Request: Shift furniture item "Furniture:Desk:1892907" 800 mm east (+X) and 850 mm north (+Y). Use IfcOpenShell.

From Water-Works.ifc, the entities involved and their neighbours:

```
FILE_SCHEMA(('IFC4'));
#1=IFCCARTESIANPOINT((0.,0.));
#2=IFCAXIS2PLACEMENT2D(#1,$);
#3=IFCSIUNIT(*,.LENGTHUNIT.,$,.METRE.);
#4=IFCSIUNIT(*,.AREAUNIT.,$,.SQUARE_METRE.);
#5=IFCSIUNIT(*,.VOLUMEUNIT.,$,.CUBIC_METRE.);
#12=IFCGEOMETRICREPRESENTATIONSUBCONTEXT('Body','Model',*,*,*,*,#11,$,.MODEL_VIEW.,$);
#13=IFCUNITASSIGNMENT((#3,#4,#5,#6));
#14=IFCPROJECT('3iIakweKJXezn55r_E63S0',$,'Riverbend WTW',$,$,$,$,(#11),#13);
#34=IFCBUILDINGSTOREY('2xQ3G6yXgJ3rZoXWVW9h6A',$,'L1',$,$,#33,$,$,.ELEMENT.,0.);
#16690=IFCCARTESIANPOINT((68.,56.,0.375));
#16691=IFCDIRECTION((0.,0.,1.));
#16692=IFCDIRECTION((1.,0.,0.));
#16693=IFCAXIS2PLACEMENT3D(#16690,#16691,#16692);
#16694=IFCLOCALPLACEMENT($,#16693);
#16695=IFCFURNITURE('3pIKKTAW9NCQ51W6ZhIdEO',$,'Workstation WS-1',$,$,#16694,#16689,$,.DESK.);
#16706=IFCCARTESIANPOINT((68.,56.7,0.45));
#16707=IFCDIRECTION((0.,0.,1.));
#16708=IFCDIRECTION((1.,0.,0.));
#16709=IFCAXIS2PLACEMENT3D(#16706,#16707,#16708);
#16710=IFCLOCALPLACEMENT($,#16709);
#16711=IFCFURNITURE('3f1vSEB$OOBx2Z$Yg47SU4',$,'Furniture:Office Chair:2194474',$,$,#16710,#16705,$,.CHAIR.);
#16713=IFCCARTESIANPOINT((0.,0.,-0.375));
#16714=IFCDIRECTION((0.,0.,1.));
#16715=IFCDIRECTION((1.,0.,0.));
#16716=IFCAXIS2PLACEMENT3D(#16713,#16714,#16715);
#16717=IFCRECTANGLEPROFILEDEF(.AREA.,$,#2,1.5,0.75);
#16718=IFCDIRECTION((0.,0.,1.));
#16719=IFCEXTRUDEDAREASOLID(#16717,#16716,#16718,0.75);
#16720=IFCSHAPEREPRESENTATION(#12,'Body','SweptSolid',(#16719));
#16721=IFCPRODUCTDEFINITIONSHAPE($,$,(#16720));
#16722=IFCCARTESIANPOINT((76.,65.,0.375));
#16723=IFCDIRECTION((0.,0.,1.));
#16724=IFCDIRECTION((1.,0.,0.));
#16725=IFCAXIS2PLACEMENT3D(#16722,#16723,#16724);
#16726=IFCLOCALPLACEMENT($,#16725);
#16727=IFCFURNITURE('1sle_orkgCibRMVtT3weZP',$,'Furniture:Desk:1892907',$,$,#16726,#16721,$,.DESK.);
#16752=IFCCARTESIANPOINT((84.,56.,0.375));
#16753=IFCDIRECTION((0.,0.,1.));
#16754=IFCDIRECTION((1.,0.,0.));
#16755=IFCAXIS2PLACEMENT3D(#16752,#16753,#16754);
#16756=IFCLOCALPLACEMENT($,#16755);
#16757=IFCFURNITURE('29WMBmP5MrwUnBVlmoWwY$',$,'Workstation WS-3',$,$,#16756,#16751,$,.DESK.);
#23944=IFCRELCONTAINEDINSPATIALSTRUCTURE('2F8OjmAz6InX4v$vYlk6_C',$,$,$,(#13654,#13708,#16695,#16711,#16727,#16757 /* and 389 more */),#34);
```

```python
import ifcopenshell
import ifcopenshell.api.geometry
import ifcopenshell.util.placement
import ifcopenshell.util.unit

model = ifcopenshell.open("Water-Works.ifc")
unit_scale = ifcopenshell.util.unit.calculate_unit_scale(model)

item = model.by_guid("1sle_orkgCibRMVtT3weZP")
matrix = ifcopenshell.util.placement.get_local_placement(item.ObjectPlacement)
matrix[0, 3] += 0.8 / unit_scale
matrix[1, 3] += 0.85 / unit_scale
ifcopenshell.api.geometry.edit_object_placement(model, product=item, matrix=matrix, is_si=False)

print(ifcopenshell.util.placement.get_local_placement(item.ObjectPlacement).round(3) + 0.0)

model.write("Water-Works_updated.ifc")
```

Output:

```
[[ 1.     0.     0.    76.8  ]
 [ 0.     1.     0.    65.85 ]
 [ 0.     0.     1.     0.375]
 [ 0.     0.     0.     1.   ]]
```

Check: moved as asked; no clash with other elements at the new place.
